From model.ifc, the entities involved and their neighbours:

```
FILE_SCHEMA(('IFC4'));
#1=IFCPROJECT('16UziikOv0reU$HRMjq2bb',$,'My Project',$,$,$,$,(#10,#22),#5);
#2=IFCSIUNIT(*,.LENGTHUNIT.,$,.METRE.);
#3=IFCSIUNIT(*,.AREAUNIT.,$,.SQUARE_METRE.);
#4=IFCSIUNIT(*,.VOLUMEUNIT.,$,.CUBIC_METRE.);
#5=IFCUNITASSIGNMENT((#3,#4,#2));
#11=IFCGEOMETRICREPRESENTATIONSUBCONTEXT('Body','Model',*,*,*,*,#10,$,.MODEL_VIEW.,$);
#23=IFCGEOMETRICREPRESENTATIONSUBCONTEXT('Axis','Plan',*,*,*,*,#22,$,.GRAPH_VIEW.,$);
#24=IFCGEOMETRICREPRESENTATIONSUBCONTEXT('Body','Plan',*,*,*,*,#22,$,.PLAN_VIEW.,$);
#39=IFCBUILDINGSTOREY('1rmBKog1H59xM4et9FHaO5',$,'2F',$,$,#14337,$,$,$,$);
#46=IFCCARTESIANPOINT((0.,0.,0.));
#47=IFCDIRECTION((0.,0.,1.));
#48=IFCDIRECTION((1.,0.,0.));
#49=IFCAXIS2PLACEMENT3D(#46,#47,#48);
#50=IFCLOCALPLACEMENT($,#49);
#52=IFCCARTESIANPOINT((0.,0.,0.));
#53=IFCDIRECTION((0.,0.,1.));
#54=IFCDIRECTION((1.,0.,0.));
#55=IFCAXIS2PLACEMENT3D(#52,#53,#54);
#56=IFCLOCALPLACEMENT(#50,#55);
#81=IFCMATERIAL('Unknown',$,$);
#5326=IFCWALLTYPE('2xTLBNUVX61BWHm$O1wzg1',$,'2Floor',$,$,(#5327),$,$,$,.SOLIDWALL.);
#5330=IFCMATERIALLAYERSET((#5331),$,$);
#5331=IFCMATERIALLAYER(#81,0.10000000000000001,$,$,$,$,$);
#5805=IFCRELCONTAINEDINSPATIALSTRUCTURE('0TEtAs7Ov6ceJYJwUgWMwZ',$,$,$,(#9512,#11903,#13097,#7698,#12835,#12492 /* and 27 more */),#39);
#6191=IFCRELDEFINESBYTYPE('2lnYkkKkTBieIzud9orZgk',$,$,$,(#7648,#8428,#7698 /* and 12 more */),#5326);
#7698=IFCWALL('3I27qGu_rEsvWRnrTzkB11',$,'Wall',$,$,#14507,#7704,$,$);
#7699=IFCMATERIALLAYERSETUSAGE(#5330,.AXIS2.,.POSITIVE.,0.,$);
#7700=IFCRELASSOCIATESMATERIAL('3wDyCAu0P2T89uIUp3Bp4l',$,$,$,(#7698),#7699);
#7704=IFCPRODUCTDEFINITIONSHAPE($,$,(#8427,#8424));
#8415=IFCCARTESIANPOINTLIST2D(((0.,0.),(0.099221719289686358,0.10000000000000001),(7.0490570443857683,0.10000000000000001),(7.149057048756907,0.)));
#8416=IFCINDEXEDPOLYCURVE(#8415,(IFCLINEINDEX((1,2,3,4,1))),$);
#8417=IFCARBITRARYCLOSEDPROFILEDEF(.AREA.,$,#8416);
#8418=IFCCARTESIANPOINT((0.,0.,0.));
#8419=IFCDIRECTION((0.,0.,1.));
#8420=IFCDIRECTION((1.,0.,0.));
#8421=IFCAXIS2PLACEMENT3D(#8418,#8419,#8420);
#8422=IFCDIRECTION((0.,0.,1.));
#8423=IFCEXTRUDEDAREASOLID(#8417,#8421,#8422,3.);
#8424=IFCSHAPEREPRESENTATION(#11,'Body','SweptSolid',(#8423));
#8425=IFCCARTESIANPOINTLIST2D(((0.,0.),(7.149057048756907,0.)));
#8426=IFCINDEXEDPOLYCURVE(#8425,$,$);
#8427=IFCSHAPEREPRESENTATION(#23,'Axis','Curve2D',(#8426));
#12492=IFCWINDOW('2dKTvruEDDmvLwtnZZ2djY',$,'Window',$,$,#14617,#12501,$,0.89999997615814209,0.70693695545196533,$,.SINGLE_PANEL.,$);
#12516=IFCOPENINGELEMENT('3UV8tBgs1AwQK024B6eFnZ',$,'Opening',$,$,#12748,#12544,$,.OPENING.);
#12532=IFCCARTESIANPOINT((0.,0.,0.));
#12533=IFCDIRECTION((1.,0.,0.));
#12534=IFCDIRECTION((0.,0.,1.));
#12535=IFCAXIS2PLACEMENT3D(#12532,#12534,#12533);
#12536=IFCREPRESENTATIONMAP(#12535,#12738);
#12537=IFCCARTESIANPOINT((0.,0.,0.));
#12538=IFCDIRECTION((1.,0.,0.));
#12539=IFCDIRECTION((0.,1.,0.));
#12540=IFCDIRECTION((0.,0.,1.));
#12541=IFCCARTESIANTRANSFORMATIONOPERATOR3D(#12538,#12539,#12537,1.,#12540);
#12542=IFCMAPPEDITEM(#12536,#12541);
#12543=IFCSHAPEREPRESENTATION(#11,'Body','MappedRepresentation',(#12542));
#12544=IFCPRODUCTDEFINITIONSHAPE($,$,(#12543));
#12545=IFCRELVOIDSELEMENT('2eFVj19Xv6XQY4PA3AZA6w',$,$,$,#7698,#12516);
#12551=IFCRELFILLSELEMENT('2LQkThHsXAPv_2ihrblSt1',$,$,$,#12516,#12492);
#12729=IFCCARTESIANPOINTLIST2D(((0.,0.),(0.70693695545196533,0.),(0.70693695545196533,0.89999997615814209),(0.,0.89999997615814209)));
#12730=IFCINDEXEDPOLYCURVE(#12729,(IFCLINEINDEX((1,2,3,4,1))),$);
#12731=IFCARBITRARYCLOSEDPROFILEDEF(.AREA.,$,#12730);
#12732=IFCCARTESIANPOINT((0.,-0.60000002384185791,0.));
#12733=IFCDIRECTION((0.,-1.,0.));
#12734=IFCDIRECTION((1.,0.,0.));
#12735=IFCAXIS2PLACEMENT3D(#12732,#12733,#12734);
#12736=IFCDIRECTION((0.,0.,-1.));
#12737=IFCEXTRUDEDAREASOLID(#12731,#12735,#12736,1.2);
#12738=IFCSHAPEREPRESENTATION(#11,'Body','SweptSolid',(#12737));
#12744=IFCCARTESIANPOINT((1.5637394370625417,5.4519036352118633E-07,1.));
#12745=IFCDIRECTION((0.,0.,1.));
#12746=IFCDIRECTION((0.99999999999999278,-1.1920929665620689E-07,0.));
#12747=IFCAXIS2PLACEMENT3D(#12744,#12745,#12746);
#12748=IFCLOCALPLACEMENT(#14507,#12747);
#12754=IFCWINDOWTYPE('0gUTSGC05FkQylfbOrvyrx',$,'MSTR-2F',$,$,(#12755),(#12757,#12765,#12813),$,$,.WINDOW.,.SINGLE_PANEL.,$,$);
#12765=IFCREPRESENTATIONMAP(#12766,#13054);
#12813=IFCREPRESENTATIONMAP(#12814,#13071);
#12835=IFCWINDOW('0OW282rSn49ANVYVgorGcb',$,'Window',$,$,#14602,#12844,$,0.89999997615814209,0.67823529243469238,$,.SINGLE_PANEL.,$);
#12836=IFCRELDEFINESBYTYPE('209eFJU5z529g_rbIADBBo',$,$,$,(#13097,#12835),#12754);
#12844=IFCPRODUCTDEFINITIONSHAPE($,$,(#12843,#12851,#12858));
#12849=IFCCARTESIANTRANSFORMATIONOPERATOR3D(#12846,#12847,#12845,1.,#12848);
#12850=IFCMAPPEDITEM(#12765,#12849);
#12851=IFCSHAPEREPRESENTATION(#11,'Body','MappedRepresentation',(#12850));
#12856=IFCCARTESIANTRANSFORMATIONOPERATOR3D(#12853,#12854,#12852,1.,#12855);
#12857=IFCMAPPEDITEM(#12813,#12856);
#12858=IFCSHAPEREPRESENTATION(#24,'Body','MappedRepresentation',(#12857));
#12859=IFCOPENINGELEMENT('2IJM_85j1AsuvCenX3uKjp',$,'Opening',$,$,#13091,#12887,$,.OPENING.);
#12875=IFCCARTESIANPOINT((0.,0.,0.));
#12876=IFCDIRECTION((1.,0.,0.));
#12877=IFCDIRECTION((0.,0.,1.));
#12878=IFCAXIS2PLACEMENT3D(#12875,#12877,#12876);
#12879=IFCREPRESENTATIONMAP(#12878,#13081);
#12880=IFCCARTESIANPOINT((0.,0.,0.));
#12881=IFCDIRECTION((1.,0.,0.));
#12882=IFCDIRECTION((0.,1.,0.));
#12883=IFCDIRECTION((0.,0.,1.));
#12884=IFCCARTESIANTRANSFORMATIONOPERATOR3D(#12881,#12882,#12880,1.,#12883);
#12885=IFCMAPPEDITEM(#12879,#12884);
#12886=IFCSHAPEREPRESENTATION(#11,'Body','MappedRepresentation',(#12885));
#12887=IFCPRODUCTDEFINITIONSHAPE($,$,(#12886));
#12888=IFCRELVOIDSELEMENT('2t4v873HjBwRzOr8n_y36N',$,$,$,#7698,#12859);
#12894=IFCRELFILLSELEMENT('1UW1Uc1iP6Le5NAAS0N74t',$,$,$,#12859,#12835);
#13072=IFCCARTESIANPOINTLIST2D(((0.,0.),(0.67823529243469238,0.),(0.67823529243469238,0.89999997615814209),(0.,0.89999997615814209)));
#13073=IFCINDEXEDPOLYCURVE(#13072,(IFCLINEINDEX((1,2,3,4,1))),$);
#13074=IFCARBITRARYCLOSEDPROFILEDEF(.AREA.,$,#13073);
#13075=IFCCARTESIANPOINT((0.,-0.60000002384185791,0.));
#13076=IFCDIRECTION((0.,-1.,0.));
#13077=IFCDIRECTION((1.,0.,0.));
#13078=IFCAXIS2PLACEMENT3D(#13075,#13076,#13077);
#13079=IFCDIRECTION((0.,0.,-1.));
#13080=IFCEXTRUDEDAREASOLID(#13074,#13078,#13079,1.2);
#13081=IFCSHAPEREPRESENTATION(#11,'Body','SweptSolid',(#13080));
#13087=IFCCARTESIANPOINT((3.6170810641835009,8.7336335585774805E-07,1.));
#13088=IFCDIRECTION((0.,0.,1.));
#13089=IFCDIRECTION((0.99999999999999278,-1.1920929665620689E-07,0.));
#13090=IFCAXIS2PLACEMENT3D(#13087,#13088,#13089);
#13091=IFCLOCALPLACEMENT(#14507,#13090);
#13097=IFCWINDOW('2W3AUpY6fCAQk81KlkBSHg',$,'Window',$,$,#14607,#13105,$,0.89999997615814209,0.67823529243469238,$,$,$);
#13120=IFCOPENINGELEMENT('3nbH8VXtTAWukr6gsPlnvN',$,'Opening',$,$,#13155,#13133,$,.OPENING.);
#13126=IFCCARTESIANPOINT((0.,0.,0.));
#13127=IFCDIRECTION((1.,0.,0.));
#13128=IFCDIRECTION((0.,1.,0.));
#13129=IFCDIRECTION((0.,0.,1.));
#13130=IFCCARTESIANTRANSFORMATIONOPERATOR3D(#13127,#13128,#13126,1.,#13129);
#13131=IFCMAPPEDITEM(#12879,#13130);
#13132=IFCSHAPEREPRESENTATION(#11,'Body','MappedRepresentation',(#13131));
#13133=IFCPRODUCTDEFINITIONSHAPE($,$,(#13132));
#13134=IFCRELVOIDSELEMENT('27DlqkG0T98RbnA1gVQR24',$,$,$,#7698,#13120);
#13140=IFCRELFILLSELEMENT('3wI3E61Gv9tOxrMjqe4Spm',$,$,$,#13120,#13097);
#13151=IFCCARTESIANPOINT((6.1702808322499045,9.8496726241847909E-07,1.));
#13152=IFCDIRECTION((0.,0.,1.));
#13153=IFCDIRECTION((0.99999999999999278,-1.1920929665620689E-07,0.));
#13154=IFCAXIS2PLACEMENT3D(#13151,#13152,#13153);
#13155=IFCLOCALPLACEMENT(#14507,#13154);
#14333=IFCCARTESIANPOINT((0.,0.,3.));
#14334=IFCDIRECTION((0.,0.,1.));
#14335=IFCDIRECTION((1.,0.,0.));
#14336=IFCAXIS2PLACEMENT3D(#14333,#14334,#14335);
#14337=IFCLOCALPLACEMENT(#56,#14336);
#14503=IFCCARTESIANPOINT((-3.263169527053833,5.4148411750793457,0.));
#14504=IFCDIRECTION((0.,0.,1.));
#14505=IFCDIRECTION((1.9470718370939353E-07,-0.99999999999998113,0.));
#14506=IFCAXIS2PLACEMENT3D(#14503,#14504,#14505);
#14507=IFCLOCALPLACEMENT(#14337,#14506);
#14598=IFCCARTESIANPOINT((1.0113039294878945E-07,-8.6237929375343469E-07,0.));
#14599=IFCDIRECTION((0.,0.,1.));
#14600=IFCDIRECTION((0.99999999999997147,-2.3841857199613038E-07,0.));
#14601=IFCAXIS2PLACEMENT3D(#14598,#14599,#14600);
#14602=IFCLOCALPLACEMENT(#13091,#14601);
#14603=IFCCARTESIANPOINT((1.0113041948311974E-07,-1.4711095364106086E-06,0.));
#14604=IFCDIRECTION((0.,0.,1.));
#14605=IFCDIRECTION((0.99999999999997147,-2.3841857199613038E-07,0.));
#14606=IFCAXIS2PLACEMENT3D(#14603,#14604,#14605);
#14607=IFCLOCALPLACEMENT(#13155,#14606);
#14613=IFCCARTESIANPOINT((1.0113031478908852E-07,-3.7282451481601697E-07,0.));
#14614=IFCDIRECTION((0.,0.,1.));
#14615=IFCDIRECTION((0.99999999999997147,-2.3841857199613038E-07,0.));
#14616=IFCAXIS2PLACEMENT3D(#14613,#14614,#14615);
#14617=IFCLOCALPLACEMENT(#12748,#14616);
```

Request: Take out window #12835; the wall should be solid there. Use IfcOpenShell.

```python
import ifcopenshell
import ifcopenshell.api.feature
import ifcopenshell.api.root
import ifcopenshell.geom
import ifcopenshell.util.shape

model = ifcopenshell.open("model.ifc")
settings = ifcopenshell.geom.settings()


def volume(element):
    """Net volume in cubic metres, openings subtracted."""
    shape = ifcopenshell.geom.create_shape(settings, element)
    return ifcopenshell.util.shape.get_volume(shape.geometry)


window = model.by_guid("0OW282rSn49ANVYVgorGcb")
opening = window.FillsVoids[0].RelatingOpeningElement
wall = opening.VoidsElements[0].RelatingBuildingElement
before = volume(wall)

ifcopenshell.api.root.remove_product(model, product=window)
ifcopenshell.api.feature.remove_feature(model, feature=opening)

after = volume(wall)

print(f"wall volume {before:.3f} -> {after:.3f} m3")

model.write("model_updated.ifc")
```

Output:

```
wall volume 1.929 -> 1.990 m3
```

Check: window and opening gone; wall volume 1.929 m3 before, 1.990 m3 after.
